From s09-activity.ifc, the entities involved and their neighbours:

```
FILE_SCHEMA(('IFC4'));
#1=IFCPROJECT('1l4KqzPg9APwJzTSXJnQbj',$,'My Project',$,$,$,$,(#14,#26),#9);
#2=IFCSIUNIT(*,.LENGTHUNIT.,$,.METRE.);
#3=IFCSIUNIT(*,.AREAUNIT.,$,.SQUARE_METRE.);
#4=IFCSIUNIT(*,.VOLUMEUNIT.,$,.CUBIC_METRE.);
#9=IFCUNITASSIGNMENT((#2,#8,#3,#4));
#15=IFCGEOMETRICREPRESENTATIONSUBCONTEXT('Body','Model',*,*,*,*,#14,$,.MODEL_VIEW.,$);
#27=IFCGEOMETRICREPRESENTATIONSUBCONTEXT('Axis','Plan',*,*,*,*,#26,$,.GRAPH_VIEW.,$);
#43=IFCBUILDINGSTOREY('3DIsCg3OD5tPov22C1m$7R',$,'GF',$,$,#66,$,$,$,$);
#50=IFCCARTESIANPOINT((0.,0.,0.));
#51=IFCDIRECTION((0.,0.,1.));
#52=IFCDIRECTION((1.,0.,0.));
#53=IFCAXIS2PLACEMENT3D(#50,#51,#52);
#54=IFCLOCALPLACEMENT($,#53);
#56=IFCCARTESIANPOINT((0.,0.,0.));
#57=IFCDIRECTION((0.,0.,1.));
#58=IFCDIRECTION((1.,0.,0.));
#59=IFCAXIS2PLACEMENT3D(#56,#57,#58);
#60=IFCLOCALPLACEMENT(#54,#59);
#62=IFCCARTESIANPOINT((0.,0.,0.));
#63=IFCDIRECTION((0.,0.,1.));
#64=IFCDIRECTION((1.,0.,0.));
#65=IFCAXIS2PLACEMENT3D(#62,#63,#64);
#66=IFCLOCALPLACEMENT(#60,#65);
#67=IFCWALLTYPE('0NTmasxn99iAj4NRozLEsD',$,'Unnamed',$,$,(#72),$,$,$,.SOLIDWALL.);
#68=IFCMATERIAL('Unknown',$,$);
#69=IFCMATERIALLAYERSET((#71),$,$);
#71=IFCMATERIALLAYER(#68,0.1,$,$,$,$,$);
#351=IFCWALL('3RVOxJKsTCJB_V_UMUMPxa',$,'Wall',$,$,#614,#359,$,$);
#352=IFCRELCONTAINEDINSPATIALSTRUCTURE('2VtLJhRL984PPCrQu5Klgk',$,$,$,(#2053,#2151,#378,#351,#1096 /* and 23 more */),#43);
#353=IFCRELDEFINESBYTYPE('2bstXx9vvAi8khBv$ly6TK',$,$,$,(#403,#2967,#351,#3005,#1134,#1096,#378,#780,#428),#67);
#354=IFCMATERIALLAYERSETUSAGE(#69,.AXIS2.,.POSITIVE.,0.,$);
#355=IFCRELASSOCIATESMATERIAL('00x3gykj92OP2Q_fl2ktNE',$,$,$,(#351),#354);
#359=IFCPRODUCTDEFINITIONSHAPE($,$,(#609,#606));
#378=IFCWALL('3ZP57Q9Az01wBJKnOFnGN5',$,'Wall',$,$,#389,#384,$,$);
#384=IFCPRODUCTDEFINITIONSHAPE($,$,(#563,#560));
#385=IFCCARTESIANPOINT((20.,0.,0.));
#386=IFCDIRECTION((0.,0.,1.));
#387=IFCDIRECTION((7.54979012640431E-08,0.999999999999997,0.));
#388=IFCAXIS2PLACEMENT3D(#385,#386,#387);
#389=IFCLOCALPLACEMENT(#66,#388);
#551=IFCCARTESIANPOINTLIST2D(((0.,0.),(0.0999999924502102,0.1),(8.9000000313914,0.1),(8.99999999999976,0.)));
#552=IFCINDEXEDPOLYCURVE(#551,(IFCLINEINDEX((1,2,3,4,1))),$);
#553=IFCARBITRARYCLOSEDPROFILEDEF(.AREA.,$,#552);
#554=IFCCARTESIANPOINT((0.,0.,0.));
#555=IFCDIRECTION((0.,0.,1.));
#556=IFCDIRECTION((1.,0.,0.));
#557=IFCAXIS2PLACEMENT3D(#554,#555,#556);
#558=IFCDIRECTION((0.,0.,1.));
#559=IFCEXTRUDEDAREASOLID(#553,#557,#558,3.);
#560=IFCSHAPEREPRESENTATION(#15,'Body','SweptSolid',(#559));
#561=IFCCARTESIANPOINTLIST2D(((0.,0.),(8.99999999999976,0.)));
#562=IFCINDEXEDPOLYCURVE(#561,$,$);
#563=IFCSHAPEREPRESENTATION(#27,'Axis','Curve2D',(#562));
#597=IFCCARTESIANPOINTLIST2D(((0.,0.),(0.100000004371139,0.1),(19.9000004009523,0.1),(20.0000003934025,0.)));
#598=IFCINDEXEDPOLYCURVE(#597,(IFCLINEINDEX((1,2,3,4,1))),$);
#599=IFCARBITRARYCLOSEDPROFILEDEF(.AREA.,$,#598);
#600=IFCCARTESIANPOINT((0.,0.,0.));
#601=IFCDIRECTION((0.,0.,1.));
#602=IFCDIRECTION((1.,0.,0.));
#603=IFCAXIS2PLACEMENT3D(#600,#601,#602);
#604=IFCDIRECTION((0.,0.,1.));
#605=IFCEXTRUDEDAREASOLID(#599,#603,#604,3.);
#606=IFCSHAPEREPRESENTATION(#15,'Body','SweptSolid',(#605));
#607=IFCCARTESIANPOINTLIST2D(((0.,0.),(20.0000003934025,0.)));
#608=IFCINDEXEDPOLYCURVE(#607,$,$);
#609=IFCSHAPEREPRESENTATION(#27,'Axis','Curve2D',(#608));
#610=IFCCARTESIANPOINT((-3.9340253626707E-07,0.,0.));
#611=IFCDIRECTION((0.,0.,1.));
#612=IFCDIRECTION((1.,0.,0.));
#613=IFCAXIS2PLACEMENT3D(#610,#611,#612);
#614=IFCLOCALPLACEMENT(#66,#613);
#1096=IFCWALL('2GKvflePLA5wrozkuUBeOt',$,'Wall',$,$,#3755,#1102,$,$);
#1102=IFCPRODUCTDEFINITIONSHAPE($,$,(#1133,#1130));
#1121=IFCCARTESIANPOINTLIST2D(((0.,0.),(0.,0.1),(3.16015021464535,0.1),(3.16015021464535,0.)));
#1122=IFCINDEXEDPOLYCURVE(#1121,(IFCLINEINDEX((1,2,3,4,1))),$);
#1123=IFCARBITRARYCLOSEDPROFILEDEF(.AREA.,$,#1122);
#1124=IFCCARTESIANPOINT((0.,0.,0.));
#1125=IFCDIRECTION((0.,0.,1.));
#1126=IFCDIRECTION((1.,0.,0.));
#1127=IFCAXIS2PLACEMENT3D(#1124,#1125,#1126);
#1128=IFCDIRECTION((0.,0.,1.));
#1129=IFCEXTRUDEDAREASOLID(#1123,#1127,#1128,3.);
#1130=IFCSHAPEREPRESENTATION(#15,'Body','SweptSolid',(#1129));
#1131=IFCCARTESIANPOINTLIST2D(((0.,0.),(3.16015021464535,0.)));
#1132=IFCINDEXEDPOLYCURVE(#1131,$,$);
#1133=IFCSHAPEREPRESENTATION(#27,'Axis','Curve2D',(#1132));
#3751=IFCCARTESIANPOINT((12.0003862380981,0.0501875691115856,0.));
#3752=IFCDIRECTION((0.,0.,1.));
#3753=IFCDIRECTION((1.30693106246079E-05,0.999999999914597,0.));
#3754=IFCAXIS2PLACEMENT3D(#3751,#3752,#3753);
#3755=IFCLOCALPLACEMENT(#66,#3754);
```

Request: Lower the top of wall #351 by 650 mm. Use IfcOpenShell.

```python
import ifcopenshell
import ifcopenshell.geom
import ifcopenshell.util.representation
import ifcopenshell.util.shape
import ifcopenshell.util.unit

model = ifcopenshell.open("s09-activity.ifc")
unit_scale = ifcopenshell.util.unit.calculate_unit_scale(model)
settings = ifcopenshell.geom.settings()


def volume(element):
    """Net volume in cubic metres, openings subtracted."""
    shape = ifcopenshell.geom.create_shape(settings, element)
    return ifcopenshell.util.shape.get_volume(shape.geometry)


wall = model.by_id(351)
before = volume(wall)

body = ifcopenshell.util.representation.get_representation(wall, "Model", "Body")
solid = body.Items[0]
old_height = solid.Depth
solid.Depth -= 0.65 / unit_scale
after = volume(wall)

print(f"height {old_height:g} -> {solid.Depth:g}, volume {before:.3f} -> {after:.3f} m3")

model.write("s09-activity_updated.ifc")
```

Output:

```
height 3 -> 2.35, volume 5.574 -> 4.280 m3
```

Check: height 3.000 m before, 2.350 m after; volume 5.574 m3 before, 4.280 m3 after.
